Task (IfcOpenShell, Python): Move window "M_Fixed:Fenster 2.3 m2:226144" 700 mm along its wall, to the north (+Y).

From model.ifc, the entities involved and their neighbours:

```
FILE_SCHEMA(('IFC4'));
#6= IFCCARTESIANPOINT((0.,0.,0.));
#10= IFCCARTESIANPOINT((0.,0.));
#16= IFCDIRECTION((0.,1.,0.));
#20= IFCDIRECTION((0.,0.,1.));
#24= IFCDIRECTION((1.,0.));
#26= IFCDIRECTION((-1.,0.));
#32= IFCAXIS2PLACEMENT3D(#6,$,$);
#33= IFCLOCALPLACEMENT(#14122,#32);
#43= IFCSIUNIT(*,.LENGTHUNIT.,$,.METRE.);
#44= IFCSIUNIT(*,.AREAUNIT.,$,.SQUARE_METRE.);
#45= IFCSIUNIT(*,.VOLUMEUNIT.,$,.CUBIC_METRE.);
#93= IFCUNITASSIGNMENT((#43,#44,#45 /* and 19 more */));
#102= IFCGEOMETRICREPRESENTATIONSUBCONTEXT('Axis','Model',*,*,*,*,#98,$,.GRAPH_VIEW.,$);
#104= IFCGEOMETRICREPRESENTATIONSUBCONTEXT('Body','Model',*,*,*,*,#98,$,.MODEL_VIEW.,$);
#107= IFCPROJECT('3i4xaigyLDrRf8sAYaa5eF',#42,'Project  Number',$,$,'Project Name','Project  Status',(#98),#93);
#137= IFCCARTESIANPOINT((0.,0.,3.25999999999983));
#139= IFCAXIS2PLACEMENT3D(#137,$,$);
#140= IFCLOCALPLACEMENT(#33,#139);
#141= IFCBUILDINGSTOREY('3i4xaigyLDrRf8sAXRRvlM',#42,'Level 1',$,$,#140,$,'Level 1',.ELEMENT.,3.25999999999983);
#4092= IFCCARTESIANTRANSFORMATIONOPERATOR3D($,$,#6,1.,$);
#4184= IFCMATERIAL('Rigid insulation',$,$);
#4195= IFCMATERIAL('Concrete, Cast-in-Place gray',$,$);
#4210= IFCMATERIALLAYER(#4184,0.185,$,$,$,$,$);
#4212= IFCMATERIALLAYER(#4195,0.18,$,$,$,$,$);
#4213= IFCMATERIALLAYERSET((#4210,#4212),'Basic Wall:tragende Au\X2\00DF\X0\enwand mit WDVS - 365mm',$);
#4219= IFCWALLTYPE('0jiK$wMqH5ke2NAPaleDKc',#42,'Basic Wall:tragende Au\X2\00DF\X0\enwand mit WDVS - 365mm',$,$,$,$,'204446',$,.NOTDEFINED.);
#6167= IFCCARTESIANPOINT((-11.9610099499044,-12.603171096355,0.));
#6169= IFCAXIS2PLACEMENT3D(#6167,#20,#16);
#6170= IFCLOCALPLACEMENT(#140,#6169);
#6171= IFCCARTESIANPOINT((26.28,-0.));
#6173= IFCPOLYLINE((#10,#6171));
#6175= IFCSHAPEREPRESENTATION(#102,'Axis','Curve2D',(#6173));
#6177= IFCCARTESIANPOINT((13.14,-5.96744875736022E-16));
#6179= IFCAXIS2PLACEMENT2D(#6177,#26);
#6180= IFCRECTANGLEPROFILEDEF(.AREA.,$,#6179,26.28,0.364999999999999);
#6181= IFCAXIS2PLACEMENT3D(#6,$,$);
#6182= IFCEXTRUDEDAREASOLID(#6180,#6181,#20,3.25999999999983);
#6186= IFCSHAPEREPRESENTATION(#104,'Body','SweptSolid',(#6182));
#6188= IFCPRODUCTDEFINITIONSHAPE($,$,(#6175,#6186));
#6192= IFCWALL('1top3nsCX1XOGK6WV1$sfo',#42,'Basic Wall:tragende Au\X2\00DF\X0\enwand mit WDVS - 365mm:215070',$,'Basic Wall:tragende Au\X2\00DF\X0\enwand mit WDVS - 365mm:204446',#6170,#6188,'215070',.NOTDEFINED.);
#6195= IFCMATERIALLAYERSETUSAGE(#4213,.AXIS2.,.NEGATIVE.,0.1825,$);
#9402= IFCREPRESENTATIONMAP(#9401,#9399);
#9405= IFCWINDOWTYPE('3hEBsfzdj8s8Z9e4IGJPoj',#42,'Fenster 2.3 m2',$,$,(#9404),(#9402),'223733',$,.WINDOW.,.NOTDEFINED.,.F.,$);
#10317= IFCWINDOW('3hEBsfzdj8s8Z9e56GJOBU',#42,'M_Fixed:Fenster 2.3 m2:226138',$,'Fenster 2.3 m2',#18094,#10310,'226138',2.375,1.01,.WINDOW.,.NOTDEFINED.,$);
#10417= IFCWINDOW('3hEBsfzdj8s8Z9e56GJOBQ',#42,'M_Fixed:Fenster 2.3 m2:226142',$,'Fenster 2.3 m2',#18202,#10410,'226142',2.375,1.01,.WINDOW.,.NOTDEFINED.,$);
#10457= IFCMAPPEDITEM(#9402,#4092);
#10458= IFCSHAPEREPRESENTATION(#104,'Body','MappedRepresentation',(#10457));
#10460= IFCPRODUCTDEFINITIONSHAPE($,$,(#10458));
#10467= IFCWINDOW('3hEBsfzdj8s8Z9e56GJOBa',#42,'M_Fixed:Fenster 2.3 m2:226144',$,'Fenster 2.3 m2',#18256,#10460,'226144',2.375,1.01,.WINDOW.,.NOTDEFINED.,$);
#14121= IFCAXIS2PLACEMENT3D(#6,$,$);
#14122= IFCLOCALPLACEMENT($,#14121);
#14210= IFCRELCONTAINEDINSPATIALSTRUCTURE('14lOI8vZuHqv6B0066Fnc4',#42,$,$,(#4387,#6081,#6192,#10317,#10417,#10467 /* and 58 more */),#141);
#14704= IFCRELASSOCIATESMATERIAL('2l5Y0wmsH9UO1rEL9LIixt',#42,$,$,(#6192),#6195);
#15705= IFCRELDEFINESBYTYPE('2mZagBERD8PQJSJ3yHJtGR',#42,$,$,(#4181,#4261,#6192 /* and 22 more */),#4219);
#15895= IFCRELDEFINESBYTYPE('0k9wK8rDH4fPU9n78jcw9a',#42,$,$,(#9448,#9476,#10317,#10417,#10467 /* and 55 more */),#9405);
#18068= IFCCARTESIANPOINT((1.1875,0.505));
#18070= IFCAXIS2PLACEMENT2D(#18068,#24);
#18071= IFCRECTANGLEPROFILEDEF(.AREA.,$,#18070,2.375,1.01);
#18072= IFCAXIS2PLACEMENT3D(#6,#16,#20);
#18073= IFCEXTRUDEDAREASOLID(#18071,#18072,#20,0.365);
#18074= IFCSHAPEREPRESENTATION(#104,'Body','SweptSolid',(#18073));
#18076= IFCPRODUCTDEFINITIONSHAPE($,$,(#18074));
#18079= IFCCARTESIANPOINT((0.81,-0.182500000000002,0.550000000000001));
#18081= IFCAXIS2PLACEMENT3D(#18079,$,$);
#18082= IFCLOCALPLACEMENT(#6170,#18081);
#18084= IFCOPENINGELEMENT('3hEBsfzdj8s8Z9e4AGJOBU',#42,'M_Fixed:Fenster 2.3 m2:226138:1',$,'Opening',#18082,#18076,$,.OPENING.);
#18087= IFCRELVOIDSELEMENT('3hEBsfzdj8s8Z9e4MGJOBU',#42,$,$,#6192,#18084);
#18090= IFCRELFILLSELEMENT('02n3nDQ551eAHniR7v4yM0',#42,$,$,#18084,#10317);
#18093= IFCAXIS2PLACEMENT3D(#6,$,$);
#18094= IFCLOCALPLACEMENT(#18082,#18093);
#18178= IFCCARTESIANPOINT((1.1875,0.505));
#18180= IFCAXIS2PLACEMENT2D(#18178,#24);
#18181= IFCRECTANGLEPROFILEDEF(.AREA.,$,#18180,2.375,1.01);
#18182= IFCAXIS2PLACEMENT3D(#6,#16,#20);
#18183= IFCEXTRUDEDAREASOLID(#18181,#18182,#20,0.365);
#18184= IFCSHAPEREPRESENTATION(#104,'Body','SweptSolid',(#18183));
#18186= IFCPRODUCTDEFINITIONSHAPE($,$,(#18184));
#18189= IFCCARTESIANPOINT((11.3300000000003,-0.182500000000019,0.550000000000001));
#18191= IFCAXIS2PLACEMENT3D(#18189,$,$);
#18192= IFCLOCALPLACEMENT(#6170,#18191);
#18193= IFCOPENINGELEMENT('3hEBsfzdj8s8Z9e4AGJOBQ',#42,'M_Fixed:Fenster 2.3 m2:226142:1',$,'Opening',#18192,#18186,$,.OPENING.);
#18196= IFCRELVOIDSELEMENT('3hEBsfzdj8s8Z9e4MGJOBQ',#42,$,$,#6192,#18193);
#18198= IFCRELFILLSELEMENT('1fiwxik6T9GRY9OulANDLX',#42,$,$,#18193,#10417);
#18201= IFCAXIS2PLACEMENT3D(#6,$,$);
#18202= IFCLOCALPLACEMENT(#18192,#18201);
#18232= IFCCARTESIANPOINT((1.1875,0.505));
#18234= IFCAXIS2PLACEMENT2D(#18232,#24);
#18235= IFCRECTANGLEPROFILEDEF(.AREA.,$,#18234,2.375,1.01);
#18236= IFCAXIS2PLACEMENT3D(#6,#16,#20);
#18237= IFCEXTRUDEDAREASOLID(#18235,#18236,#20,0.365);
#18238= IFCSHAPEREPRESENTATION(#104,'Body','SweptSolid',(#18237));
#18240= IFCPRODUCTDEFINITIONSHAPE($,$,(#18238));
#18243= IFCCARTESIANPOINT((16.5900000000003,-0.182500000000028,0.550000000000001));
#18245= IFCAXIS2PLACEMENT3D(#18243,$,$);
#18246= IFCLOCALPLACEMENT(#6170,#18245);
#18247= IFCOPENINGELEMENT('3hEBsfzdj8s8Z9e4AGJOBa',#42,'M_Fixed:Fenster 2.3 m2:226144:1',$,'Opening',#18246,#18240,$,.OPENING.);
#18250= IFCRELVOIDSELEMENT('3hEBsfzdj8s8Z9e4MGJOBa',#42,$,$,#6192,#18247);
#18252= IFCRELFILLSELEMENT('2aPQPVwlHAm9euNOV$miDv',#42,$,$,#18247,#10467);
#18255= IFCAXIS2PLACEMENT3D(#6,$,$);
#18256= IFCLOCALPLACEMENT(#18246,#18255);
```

```python
import ifcopenshell
import ifcopenshell.api.geometry
import ifcopenshell.util.placement

model = ifcopenshell.open("model.ifc")

window = model.by_guid("3hEBsfzdj8s8Z9e56GJOBa")
opening = window.FillsVoids[0].RelatingOpeningElement
wall = opening.VoidsElements[0].RelatingBuildingElement

wall_matrix = ifcopenshell.util.placement.get_local_placement(wall.ObjectPlacement)
shift = wall_matrix[:3, 0] * 0.7
before = ifcopenshell.util.placement.get_local_placement(window.ObjectPlacement)[:3, 3].copy()

# The window is placed relative to its opening, so it follows when the opening moves.
matrix = ifcopenshell.util.placement.get_local_placement(opening.ObjectPlacement)
matrix[:3, 3] += shift
ifcopenshell.api.geometry.edit_object_placement(
    model, product=opening, matrix=matrix, is_si=False, should_transform_children=True
)

after = ifcopenshell.util.placement.get_local_placement(window.ObjectPlacement)[:3, 3]
print("window moved by", (after - before).round(3) + 0.0)

model.write("model_v2.ifc")
```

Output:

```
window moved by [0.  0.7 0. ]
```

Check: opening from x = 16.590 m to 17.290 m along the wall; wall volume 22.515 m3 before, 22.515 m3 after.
